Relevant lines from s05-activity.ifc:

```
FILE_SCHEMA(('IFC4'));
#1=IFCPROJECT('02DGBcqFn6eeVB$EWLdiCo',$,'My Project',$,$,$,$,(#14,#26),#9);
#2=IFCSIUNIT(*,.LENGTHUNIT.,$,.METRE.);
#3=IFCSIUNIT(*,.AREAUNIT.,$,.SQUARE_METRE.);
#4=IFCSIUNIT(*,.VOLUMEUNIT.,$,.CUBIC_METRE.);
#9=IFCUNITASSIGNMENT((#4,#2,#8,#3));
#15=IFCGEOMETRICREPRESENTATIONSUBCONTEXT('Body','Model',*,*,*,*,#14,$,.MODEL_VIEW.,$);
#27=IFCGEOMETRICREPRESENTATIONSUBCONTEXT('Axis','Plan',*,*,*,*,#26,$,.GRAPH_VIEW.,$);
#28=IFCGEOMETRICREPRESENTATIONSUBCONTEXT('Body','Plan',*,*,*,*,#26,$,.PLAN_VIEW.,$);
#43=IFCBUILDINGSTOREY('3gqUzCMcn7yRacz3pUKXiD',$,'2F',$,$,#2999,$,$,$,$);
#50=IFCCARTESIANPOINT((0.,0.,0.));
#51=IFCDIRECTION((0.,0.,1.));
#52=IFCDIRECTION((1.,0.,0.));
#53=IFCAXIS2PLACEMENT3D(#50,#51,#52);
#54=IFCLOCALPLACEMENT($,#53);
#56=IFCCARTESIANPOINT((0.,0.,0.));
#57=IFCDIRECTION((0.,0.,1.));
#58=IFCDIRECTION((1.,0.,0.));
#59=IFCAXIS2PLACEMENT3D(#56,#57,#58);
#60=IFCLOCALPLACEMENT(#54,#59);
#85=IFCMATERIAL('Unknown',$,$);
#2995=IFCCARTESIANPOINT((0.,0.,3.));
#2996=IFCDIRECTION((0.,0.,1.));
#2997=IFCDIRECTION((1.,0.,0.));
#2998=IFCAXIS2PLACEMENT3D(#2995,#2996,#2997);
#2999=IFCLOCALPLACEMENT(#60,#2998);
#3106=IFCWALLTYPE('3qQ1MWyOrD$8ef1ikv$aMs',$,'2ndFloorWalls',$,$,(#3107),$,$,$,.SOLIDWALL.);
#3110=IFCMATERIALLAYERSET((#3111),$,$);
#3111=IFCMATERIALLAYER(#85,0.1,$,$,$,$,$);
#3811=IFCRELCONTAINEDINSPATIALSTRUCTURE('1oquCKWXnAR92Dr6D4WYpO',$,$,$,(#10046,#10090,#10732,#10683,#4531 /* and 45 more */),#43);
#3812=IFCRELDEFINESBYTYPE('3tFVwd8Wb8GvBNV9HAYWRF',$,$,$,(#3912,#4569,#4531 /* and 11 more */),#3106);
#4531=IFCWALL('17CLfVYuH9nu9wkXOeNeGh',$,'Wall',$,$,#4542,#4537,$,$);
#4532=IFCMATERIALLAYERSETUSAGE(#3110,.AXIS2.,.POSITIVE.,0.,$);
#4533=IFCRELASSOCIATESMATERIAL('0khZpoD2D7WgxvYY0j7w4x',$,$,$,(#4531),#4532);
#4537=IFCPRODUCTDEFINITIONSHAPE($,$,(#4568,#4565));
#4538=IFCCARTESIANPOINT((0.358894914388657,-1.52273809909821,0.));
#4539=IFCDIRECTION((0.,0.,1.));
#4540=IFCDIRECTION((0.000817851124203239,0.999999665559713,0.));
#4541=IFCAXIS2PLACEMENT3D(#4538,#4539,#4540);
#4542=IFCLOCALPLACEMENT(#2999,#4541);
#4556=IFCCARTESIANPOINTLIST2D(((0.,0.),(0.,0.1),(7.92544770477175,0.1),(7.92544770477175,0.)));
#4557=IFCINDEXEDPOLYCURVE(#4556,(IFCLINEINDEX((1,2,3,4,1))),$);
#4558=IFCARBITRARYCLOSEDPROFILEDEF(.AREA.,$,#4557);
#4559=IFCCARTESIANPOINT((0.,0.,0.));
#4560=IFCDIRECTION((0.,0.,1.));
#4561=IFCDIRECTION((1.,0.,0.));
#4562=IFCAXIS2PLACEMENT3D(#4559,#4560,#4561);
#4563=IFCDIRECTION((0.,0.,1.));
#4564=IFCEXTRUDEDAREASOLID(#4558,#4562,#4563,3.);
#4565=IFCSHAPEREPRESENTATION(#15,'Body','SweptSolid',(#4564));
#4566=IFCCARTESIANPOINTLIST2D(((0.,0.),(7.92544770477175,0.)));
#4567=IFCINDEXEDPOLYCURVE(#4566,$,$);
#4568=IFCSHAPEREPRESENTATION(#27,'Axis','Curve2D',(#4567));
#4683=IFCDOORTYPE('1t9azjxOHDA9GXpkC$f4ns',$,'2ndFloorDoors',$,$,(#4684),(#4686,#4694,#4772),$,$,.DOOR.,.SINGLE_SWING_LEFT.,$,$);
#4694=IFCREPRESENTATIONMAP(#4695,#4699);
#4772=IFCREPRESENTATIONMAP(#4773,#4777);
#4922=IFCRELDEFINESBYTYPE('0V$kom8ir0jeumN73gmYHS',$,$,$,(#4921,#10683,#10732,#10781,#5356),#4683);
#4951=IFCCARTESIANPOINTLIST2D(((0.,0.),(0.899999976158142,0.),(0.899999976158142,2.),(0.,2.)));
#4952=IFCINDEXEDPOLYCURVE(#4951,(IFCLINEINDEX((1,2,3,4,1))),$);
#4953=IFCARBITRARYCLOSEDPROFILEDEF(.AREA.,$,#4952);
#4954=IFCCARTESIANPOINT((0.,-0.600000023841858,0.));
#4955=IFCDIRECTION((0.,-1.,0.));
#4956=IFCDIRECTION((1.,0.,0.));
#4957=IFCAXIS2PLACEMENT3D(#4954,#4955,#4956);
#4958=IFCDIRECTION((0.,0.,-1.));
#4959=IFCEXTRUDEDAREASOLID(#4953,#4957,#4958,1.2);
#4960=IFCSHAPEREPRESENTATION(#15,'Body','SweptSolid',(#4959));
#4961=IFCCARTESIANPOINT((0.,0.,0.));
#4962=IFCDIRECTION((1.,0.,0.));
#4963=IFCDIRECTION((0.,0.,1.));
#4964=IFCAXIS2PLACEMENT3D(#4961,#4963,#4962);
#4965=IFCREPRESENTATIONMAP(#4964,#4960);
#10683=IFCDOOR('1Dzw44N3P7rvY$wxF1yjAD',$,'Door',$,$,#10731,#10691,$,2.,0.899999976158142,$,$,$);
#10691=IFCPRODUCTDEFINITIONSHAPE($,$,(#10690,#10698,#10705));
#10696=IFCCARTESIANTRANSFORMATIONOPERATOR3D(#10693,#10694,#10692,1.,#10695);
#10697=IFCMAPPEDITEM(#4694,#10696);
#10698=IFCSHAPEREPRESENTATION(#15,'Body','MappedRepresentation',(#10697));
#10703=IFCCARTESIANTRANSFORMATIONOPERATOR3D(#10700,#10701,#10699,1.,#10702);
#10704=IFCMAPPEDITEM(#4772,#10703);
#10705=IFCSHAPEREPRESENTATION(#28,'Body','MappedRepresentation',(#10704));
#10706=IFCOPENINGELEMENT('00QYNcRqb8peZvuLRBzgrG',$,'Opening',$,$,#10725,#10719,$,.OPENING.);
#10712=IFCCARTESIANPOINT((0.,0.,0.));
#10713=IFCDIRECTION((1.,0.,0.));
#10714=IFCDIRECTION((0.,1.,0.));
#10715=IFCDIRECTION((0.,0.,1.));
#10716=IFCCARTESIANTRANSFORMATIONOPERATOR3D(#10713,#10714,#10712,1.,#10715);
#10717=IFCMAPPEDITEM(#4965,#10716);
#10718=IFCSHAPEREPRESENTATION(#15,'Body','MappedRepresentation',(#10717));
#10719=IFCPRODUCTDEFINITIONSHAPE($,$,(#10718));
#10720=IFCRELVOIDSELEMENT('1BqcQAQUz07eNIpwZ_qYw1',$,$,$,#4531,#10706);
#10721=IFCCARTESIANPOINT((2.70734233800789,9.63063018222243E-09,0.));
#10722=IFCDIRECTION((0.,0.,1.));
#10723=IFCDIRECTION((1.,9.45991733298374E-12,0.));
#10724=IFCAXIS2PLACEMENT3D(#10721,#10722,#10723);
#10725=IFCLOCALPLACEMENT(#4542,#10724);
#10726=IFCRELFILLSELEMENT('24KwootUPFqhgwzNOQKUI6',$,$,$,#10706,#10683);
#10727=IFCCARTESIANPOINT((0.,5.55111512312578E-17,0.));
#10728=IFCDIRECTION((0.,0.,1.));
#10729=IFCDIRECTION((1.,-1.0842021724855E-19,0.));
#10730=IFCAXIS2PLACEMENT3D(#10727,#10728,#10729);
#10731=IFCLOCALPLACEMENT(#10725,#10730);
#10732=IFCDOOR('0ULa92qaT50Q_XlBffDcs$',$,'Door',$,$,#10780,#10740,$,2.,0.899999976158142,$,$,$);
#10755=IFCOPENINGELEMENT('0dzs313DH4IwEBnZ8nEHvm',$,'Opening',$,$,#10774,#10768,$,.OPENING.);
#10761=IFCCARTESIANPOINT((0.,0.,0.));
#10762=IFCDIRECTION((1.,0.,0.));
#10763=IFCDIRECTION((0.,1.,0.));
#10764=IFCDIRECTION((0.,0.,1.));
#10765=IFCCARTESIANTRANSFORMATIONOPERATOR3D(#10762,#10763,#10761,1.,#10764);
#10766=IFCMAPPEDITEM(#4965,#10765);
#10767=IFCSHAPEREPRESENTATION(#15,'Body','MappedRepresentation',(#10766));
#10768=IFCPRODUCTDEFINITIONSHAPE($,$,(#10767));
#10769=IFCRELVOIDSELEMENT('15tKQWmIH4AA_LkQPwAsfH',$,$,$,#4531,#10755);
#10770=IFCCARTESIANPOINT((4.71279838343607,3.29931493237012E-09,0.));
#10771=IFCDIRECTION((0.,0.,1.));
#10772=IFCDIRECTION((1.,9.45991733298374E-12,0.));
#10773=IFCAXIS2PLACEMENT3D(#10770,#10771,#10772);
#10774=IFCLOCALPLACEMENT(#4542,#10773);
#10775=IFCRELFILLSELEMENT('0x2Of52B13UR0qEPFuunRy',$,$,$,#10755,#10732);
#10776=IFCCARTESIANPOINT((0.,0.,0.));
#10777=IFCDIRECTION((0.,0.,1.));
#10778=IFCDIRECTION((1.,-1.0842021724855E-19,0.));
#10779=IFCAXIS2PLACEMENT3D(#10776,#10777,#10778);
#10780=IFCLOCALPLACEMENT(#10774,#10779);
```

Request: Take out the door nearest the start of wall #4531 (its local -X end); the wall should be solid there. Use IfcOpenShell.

```python
import ifcopenshell
import ifcopenshell.api.feature
import ifcopenshell.api.root
import ifcopenshell.geom
import ifcopenshell.util.shape

model = ifcopenshell.open("s05-activity.ifc")
settings = ifcopenshell.geom.settings()


def volume(element):
    """Net volume in cubic metres, openings subtracted."""
    shape = ifcopenshell.geom.create_shape(settings, element)
    return ifcopenshell.util.shape.get_volume(shape.geometry)


door = model.by_id(10683)
opening = door.FillsVoids[0].RelatingOpeningElement
wall = opening.VoidsElements[0].RelatingBuildingElement
before = volume(wall)

ifcopenshell.api.root.remove_product(model, product=door)
ifcopenshell.api.feature.remove_feature(model, feature=opening)

after = volume(wall)

print(f"wall volume {before:.3f} -> {after:.3f} m3")

model.write("s05-activity_rev.ifc")
```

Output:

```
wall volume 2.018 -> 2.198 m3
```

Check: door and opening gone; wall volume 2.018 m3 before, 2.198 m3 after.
